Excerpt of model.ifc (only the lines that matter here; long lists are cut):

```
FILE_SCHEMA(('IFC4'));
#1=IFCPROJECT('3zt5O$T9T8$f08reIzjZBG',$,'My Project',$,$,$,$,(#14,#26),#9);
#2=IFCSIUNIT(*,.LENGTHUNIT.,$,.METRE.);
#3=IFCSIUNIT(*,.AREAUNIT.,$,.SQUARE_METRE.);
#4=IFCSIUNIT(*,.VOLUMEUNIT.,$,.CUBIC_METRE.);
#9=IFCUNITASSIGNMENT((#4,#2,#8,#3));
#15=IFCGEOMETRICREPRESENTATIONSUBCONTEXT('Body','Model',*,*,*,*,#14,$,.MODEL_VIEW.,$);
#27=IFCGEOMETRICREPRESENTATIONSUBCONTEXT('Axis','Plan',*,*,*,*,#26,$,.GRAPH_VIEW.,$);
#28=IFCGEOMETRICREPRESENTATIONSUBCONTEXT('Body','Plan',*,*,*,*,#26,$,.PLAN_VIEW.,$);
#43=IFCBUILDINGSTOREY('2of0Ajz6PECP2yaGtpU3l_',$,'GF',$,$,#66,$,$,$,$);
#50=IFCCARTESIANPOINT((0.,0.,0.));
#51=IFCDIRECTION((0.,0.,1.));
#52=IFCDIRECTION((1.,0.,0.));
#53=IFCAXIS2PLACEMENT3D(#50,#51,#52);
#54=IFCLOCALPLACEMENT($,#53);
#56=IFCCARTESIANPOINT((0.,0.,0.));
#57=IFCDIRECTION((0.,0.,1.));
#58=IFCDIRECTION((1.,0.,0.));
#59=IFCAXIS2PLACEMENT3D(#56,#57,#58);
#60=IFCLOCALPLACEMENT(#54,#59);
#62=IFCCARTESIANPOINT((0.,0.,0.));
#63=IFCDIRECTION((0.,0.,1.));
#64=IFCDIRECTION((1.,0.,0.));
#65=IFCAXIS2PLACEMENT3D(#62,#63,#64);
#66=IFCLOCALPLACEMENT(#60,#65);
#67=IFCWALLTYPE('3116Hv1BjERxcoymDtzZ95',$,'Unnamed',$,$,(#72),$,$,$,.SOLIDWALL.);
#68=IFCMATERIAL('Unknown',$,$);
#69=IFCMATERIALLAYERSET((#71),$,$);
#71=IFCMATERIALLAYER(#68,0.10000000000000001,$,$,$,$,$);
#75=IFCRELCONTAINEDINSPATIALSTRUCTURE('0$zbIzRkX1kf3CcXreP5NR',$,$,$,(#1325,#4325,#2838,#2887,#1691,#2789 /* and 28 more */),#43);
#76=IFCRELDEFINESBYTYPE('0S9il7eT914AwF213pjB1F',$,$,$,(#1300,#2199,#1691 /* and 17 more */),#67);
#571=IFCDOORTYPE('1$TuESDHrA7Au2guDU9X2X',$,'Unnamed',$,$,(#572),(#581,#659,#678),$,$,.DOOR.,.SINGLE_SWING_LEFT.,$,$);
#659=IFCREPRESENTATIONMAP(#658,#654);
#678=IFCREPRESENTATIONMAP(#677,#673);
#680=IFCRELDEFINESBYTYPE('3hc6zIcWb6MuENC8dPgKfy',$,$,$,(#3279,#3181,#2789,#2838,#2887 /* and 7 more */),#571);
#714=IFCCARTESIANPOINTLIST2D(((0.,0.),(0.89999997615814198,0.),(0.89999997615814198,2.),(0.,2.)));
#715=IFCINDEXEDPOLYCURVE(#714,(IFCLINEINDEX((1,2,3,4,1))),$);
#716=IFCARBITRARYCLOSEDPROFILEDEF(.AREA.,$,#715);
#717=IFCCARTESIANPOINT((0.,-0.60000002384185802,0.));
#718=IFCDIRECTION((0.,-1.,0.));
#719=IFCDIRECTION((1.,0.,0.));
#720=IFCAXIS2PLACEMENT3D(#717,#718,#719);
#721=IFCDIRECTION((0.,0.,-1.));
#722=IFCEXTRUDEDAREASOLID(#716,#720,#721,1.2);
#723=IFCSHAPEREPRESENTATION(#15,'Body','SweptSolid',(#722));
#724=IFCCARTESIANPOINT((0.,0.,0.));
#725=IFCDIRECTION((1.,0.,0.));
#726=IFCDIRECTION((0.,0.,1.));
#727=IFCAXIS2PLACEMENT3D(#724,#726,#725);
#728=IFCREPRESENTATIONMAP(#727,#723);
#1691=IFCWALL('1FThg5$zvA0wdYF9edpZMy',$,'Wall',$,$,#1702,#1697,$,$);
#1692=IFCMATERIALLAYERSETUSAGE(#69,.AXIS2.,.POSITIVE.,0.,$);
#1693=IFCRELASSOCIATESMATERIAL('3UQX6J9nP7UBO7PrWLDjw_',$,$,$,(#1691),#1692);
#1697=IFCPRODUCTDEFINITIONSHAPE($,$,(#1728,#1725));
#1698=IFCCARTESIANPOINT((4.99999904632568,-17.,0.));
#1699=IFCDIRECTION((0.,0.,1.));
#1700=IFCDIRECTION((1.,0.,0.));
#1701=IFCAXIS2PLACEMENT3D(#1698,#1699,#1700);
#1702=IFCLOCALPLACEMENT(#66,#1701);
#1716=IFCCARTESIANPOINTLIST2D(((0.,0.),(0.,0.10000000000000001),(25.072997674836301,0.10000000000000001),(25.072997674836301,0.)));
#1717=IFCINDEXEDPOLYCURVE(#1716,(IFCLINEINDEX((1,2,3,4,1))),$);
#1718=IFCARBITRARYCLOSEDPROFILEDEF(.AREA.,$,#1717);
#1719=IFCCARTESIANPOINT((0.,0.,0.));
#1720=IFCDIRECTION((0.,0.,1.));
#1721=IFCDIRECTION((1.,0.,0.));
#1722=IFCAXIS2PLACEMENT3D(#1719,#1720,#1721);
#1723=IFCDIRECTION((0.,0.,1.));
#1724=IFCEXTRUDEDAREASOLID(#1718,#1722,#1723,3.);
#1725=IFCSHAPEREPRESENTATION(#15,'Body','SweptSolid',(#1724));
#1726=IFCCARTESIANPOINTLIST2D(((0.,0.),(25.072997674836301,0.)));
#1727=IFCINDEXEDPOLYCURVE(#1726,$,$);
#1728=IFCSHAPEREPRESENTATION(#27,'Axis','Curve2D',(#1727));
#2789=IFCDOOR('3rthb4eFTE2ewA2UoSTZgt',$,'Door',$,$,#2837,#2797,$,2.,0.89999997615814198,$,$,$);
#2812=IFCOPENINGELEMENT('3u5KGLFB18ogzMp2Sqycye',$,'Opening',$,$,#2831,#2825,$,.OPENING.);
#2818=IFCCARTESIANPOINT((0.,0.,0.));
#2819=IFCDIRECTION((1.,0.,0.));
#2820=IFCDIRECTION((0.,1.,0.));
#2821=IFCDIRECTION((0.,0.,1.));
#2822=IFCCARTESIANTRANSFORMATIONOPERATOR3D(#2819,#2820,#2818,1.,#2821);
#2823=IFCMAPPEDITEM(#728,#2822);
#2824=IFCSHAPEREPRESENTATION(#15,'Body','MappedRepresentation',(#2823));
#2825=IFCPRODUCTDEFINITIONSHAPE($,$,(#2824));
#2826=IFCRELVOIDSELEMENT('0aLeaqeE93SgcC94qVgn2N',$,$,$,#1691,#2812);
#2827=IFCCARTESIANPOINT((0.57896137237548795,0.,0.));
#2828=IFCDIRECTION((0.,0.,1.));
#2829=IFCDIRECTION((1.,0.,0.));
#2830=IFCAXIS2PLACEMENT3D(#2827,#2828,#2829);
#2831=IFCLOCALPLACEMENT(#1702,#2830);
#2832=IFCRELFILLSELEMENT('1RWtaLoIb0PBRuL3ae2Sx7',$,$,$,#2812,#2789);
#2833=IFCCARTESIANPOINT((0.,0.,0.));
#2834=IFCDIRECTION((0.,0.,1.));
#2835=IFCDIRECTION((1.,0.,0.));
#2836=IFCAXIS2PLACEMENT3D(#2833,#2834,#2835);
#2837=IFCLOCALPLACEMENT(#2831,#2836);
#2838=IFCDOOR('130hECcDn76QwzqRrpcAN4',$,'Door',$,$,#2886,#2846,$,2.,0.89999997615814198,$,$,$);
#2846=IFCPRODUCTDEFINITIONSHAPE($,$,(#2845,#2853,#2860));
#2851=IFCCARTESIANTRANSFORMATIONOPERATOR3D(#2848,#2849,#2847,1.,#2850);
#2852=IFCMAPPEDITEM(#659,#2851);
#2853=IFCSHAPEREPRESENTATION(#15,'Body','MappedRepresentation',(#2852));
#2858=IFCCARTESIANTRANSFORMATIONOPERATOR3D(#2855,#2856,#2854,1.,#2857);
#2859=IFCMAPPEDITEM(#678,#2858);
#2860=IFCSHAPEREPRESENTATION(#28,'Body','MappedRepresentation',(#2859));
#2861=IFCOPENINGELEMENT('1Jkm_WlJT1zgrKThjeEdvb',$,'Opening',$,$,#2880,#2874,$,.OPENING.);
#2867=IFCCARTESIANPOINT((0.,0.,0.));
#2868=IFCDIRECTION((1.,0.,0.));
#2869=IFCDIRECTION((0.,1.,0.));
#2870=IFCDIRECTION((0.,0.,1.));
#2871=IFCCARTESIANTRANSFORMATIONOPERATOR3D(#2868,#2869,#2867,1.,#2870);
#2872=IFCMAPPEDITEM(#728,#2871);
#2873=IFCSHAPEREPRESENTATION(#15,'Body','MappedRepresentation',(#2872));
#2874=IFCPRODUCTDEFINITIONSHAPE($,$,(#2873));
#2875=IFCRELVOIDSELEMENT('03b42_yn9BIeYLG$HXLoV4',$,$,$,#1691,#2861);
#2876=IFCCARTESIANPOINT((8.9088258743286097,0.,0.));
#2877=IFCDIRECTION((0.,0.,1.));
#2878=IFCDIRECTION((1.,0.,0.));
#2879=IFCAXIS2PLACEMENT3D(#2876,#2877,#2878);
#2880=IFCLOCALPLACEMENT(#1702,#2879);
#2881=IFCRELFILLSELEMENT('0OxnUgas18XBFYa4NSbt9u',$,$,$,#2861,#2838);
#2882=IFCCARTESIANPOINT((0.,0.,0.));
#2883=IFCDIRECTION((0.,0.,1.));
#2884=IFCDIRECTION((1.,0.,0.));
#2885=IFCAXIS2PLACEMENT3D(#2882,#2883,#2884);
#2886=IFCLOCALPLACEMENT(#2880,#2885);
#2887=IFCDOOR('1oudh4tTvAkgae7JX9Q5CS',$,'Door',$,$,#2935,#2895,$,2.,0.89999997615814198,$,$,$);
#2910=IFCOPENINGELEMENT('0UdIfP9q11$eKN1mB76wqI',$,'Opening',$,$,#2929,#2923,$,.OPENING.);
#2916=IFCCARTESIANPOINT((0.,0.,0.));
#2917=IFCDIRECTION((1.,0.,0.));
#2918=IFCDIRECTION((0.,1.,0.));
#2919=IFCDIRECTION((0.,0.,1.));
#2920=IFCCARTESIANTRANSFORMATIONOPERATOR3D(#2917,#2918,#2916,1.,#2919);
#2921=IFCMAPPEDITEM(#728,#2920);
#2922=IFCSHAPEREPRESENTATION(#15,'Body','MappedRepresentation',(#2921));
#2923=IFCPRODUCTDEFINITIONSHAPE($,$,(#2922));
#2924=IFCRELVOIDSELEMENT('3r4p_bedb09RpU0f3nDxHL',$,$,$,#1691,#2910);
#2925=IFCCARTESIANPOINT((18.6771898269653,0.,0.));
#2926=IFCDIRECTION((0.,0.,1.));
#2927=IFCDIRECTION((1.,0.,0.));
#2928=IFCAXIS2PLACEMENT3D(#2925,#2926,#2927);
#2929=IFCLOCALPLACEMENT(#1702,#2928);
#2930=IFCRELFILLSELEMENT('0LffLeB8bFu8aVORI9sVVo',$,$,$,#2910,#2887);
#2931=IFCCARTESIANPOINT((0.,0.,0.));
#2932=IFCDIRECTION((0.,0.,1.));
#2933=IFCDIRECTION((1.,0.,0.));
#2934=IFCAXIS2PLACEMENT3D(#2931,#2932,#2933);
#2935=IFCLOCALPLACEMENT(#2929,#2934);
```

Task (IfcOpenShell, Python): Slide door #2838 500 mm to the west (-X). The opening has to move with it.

```python
import ifcopenshell
import ifcopenshell.api.geometry
import ifcopenshell.util.placement

model = ifcopenshell.open("model.ifc")

door = model.by_guid("130hECcDn76QwzqRrpcAN4")
opening = door.FillsVoids[0].RelatingOpeningElement
wall = opening.VoidsElements[0].RelatingBuildingElement

wall_matrix = ifcopenshell.util.placement.get_local_placement(wall.ObjectPlacement)
shift = wall_matrix[:3, 0] * -0.5
before = ifcopenshell.util.placement.get_local_placement(door.ObjectPlacement)[:3, 3].copy()

# The door is placed relative to its opening, so it follows when the opening moves.
matrix = ifcopenshell.util.placement.get_local_placement(opening.ObjectPlacement)
matrix[:3, 3] += shift
ifcopenshell.api.geometry.edit_object_placement(
    model, product=opening, matrix=matrix, is_si=False, should_transform_children=True
)

after = ifcopenshell.util.placement.get_local_placement(door.ObjectPlacement)[:3, 3]
print("door moved by", (after - before).round(3) + 0.0)

model.write("model-out.ifc")
```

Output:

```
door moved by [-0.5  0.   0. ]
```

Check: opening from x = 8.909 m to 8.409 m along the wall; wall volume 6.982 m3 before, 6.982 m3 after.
